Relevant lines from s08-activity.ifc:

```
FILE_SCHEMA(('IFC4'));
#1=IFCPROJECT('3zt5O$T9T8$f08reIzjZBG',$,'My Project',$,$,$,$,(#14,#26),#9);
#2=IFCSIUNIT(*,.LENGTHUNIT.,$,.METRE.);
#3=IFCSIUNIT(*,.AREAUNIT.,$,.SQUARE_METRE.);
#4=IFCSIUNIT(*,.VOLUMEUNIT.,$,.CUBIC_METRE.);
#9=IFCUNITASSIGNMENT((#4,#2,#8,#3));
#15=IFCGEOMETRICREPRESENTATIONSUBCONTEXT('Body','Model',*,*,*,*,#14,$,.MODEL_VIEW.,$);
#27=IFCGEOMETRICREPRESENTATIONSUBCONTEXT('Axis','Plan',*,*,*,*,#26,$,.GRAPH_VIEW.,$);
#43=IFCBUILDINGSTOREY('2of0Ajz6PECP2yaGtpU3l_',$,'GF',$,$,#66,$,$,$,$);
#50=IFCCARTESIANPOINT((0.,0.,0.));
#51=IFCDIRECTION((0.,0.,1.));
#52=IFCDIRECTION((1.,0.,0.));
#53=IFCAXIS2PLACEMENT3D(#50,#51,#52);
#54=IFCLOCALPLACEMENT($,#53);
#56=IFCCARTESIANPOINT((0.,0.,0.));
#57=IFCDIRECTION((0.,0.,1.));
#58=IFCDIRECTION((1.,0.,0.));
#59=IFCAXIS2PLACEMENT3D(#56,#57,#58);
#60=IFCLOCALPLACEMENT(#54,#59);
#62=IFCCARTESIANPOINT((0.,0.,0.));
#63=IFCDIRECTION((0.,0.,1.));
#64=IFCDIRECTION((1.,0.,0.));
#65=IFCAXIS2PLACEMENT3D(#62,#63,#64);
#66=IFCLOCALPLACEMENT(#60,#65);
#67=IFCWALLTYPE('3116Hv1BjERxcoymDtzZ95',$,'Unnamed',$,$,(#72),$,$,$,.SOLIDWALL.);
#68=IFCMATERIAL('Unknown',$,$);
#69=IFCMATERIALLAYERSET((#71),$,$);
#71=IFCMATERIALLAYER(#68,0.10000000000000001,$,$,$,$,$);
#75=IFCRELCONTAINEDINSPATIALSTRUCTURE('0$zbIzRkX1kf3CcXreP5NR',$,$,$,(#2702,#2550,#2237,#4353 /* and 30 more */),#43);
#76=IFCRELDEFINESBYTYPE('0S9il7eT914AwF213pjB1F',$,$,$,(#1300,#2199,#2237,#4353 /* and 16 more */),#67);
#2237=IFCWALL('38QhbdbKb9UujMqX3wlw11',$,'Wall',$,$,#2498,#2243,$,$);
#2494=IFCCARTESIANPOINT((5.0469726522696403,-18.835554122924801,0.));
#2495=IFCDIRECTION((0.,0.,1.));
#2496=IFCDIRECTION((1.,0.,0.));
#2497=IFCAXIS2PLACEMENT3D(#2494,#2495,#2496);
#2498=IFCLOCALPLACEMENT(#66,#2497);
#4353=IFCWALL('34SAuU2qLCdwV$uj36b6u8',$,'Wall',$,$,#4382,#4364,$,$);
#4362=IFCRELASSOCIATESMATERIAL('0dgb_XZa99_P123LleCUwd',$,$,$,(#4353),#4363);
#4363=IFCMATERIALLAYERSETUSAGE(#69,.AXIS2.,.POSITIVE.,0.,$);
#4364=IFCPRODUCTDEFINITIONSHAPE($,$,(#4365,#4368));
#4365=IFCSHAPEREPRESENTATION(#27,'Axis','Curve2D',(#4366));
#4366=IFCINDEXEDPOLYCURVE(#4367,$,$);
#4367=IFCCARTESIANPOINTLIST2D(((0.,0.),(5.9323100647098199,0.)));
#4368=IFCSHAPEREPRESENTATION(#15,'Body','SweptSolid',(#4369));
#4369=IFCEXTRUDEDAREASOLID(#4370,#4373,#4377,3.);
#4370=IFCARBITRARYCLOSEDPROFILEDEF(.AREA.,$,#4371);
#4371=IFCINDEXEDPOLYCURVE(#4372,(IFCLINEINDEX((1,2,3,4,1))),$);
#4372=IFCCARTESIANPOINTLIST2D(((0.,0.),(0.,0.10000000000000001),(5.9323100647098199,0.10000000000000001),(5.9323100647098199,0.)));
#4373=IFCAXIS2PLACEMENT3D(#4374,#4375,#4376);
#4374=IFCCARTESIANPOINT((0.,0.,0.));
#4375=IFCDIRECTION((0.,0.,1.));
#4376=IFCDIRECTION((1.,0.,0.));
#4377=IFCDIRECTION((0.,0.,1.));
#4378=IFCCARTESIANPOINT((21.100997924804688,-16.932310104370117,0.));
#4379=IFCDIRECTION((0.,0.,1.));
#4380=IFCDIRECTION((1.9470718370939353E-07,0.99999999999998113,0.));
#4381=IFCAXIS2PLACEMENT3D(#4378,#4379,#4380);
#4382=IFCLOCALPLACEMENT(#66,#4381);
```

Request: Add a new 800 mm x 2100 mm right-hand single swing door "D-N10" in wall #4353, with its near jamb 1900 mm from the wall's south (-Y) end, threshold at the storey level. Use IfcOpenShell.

```python
import numpy as np
import ifcopenshell
import ifcopenshell.api.feature
import ifcopenshell.api.geometry
import ifcopenshell.api.root
import ifcopenshell.api.spatial
import ifcopenshell.geom
import ifcopenshell.util.element
import ifcopenshell.util.placement
import ifcopenshell.util.representation
import ifcopenshell.util.shape
import ifcopenshell.util.unit

model = ifcopenshell.open("s08-activity.ifc")
unit_scale = ifcopenshell.util.unit.calculate_unit_scale(model)
settings = ifcopenshell.geom.settings()


def volume(element):
    """Net volume in cubic metres, openings subtracted."""
    shape = ifcopenshell.geom.create_shape(settings, element)
    return ifcopenshell.util.shape.get_volume(shape.geometry)


wall = model.by_id(4353)
storey = ifcopenshell.util.element.get_container(wall, ifc_class="IfcBuildingStorey")
context = ifcopenshell.util.representation.get_context(model, "Model", "Body", "MODEL_VIEW")
before = volume(wall)

width, height, from_end, sill = 0.8, 2.1, 1.9, 0.0  # metres

# The wall runs along its own X axis, and the end named is its -X end.
wall_shape = ifcopenshell.geom.create_shape(settings, wall)
x, y, z = ifcopenshell.util.shape.get_vertices(wall_shape.geometry).T
start = x.min() + from_end
face, thickness = float(y.min()), float(y.max() - y.min())
wall_matrix = ifcopenshell.util.placement.get_local_placement(wall.ObjectPlacement)
level = ifcopenshell.util.placement.get_local_placement(storey.ObjectPlacement)[2, 3]


def in_wall(x, y):
    """Placement at x, y metres in the wall's axes, at sill height."""
    matrix = wall_matrix.copy()
    matrix[:, 3] = wall_matrix @ np.array([x / unit_scale, y / unit_scale, 0.0, 1.0])
    matrix[2, 3] = level + sill / unit_scale
    return matrix


# Opening: a box that overshoots both wall faces by 50 mm.
opening = ifcopenshell.api.root.create_entity(model, ifc_class="IfcOpeningElement", predefined_type="OPENING")
box = ifcopenshell.api.geometry.add_wall_representation(
    model, context=context, length=width, height=height, thickness=thickness + 0.1
)
ifcopenshell.api.geometry.assign_representation(model, product=opening, representation=box)
ifcopenshell.api.geometry.edit_object_placement(model, product=opening, matrix=in_wall(start, face - 0.05), is_si=False)
ifcopenshell.api.feature.add_feature(model, feature=opening, element=wall)

door = ifcopenshell.api.root.create_entity(model, ifc_class="IfcDoor", name="D-N10", predefined_type="DOOR")
door.OverallWidth, door.OverallHeight = width / unit_scale, height / unit_scale
door.OperationType = "SINGLE_SWING_RIGHT"
body = ifcopenshell.api.geometry.add_door_representation(
    model,
    context=context,
    overall_width=door.OverallWidth,
    overall_height=door.OverallHeight,
    operation_type="SINGLE_SWING_RIGHT",
    lining_properties={"LiningDepth": thickness / unit_scale, "ThresholdDepth": thickness / unit_scale},
)
ifcopenshell.api.geometry.assign_representation(model, product=door, representation=body)
ifcopenshell.api.spatial.assign_container(model, products=[door], relating_structure=storey)
ifcopenshell.api.feature.add_filling(model, opening=opening, element=door)

# The lining spans the wall, so the door starts at the wall face.
ifcopenshell.api.geometry.edit_object_placement(model, product=door, matrix=in_wall(start, face), is_si=False)

after = volume(wall)

print(f"wall volume {before:.3f} -> {after:.3f} m3")

model.write("s08-activity_edited.ifc")
```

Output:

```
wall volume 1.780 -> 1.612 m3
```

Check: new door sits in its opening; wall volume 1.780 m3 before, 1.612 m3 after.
